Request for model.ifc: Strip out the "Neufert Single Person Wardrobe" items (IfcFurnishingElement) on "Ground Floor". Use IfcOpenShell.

First a look at what the model holds.

```python
import ifcopenshell
import ifcopenshell.util.element

model = ifcopenshell.open("model.ifc")
print(model.schema)
storey = next(s for s in model.by_type("IfcBuildingStorey") if s.Name == "Ground Floor")
furniture = [e for e in ifcopenshell.util.element.get_decomposition(storey) if e.is_a("IfcFurnishingElement")]
seen = {}
for e in furniture:
    element_type = ifcopenshell.util.element.get_type(e)
    name = element_type.Name if element_type not in (None, e) else None
    seen[name] = seen.get(name, 0) + 1
for name, count in sorted(seen.items(), key=str):
    print(count, "x", name)
```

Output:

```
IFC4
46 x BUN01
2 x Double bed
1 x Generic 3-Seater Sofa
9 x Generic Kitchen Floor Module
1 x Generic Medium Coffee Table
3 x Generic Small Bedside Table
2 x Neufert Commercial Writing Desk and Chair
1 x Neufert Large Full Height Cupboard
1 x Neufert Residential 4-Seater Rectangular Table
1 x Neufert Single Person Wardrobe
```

```python
import ifcopenshell
import ifcopenshell.api.root
import ifcopenshell.util.element

model = ifcopenshell.open("model.ifc")

storey = next(s for s in model.by_type("IfcBuildingStorey") if s.Name == "Ground Floor")
furniture = [e for e in ifcopenshell.util.element.get_decomposition(storey) if e.is_a("IfcFurnishingElement")]
targets = [e for e in furniture if (t := ifcopenshell.util.element.get_type(e)) not in (None, e) and t.Name == "Neufert Single Person Wardrobe"]

for e in targets:
    ifcopenshell.api.root.remove_product(model, product=e)
print(len(targets), "removed")

model.write("model_edited.ifc")
```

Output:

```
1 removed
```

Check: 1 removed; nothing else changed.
